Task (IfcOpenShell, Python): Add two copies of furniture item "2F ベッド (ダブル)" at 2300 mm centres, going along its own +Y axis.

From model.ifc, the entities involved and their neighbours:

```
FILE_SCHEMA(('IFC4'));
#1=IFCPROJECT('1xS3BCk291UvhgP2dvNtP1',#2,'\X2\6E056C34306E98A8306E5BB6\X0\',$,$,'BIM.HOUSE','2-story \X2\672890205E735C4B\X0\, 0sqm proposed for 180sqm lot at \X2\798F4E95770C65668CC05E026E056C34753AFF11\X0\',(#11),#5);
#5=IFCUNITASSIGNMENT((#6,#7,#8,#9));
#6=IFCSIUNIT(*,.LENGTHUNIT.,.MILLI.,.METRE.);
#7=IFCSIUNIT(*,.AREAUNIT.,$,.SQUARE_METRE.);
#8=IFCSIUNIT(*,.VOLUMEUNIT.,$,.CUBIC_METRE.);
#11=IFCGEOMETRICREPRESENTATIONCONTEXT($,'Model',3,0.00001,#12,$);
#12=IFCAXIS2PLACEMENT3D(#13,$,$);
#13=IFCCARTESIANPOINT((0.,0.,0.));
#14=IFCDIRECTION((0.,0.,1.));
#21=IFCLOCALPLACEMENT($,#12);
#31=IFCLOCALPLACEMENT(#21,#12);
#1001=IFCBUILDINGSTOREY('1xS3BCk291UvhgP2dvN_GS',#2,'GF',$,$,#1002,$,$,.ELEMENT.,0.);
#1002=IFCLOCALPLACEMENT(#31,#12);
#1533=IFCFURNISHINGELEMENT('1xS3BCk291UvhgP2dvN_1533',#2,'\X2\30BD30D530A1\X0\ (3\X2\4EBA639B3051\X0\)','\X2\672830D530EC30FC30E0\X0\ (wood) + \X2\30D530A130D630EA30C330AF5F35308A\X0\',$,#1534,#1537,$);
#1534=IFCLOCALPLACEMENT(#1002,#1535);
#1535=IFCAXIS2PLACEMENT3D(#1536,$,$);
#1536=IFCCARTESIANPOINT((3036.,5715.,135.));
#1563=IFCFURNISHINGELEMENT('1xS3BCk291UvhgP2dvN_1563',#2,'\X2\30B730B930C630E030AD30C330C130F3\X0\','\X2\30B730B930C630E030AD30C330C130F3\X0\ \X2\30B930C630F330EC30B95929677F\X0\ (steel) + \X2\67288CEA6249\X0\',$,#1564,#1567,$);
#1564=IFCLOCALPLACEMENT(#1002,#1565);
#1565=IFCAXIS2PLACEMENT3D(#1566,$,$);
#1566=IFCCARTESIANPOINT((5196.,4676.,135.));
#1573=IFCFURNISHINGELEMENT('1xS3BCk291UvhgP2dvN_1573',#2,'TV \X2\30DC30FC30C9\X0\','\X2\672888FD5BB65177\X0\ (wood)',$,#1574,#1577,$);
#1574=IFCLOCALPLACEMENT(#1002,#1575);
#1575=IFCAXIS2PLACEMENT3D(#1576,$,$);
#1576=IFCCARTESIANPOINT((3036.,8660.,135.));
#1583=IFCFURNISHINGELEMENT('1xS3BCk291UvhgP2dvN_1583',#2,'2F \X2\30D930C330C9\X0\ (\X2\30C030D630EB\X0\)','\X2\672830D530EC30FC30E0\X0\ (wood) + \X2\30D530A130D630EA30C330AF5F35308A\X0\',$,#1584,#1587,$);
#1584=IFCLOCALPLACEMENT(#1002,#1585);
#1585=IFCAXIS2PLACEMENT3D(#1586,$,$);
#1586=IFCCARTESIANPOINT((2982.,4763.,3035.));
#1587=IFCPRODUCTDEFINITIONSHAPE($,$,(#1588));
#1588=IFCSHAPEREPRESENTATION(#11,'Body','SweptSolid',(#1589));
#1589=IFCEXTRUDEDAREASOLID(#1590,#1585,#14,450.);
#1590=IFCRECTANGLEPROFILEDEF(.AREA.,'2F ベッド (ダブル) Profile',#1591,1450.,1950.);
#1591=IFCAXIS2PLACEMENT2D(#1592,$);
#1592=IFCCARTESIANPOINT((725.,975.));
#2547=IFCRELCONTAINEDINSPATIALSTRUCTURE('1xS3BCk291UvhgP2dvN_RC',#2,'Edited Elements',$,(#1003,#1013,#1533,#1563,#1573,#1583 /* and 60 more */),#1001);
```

```python
import ifcopenshell
import ifcopenshell.api.geometry
import ifcopenshell.api.root
import ifcopenshell.util.element
import ifcopenshell.util.placement
import ifcopenshell.util.unit

model = ifcopenshell.open("model.ifc")
unit_scale = ifcopenshell.util.unit.calculate_unit_scale(model)


def reuse_history(source, copy):
    """copy_class also copies each property set's owner history, people and application; keep the originals."""
    for rel in copy.IsDefinedBy:
        if rel.is_a("IfcRelDefinesByProperties") and (history := rel.RelatingPropertyDefinition.OwnerHistory):
            rel.RelatingPropertyDefinition.OwnerHistory = source.OwnerHistory
            ifcopenshell.util.element.remove_deep2(model, history)


source = model.by_id(1583)
base = ifcopenshell.util.placement.get_local_placement(source.ObjectPlacement)
step = base[:3, 1] * 2.3 / unit_scale

for i in range(1, 3):
    copy = ifcopenshell.api.root.copy_class(model, product=source)
    copy.Representation = ifcopenshell.util.element.copy_deep(
        model, source.Representation, exclude=["IfcGeometricRepresentationContext", "IfcRepresentationMap"]
    )
    reuse_history(source, copy)
    matrix = base.copy()
    matrix[:3, 3] += i * step
    print("added at", matrix[:3, 3].round(3) + 0.0)
    ifcopenshell.api.geometry.edit_object_placement(model, product=copy, matrix=matrix, is_si=False)

model.write("model-out.ifc")
```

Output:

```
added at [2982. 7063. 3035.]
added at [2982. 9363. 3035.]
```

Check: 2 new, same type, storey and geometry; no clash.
